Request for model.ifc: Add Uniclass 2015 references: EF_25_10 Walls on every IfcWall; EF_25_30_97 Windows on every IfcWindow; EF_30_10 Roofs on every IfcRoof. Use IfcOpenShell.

First a look at what the model holds.

```python
import ifcopenshell

model = ifcopenshell.open("model.ifc")
print(model.schema)
print("classifications:", [c.Name for c in model.by_type("IfcClassification")])
for ifc_class in ("IfcDoor", "IfcRoof", "IfcStair", "IfcWall", "IfcWindow"):
    print(ifc_class, len(model.by_type(ifc_class)))
```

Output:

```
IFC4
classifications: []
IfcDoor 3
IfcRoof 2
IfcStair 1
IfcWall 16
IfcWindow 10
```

```python
import ifcopenshell
import ifcopenshell.api.classification

model = ifcopenshell.open("model.ifc")

system = ifcopenshell.api.classification.add_classification(model, classification="Uniclass 2015")

codes = {
    "IfcWall": ("EF_25_10", "Walls"),
    "IfcWindow": ("EF_25_30_97", "Windows"),
    "IfcRoof": ("EF_30_10", "Roofs"),
}
for ifc_class, (code, name) in codes.items():
    products = model.by_type(ifc_class)
    ifcopenshell.api.classification.add_reference(
        model, products=products, classification=system, identification=code, name=name
    )
    print(code, len(products))

model.write("model-out.ifc")
```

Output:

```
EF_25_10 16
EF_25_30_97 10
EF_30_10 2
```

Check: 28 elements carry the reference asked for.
